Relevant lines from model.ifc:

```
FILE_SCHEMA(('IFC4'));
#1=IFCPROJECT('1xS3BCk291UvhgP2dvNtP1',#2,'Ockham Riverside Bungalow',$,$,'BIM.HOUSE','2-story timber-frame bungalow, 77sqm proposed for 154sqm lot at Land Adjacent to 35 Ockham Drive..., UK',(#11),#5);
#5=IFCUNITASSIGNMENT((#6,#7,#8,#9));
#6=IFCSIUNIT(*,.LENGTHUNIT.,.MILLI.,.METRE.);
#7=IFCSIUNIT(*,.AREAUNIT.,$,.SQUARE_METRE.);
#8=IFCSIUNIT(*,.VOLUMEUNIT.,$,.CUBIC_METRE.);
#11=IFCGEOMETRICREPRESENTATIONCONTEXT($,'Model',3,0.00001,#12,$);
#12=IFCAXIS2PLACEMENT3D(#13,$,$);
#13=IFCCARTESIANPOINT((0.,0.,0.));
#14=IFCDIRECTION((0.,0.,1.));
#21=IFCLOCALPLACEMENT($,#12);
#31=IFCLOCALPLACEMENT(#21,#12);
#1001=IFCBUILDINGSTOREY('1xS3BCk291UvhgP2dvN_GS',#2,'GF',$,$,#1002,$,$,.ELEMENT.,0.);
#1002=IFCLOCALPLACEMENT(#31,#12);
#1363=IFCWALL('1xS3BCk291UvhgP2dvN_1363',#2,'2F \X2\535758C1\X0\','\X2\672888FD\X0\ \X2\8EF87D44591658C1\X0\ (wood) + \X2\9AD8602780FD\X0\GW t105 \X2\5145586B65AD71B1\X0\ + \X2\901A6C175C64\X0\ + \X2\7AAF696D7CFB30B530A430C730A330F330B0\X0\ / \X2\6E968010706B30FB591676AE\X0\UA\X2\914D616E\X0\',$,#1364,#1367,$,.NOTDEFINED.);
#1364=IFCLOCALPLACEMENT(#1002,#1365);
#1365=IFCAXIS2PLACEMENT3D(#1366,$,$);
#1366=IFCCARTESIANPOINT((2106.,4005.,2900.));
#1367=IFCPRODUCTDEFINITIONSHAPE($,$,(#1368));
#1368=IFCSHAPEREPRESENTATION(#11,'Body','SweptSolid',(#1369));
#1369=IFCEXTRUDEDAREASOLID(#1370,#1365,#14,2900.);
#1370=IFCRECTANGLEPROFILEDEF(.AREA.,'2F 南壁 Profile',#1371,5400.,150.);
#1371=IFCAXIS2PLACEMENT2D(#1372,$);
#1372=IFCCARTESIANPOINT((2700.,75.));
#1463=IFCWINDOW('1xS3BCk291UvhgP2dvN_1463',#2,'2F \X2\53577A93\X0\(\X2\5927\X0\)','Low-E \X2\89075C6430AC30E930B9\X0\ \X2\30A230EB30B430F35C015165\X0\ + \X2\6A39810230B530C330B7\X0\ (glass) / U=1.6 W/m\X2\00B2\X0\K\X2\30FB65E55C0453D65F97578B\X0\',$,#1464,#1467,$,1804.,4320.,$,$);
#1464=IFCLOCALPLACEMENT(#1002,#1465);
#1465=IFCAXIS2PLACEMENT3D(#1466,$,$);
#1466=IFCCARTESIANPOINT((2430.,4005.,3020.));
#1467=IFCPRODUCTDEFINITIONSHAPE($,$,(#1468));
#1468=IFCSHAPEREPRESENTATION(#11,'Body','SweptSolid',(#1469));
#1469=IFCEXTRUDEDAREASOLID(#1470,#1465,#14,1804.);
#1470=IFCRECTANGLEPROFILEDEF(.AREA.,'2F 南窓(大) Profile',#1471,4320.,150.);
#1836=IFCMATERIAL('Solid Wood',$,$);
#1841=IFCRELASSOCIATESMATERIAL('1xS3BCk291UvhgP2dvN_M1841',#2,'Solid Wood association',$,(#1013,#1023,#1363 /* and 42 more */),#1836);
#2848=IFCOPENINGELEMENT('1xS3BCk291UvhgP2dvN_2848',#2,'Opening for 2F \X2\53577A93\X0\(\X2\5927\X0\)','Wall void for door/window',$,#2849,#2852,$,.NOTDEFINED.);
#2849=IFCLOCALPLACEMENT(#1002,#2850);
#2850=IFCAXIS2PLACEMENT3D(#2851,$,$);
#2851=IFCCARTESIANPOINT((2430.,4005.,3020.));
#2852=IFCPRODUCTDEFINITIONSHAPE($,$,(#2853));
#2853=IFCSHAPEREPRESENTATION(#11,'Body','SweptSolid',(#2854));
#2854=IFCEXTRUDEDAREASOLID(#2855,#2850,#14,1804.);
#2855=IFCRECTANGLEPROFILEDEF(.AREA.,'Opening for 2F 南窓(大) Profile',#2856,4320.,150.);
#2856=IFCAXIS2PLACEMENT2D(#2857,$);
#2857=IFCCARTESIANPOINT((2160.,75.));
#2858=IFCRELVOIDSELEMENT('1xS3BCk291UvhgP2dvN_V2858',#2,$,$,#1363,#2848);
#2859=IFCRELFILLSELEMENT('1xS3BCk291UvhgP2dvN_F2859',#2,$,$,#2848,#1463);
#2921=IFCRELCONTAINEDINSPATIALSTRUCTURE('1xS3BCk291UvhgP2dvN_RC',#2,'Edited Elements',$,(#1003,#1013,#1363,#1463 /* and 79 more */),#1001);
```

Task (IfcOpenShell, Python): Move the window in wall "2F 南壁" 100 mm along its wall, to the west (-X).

```python
import ifcopenshell
import ifcopenshell.api.geometry
import ifcopenshell.util.placement
import ifcopenshell.util.unit

model = ifcopenshell.open("model.ifc")
unit_scale = ifcopenshell.util.unit.calculate_unit_scale(model)

window = model.by_guid("1xS3BCk291UvhgP2dvN_1463")
opening = window.FillsVoids[0].RelatingOpeningElement
wall = opening.VoidsElements[0].RelatingBuildingElement

wall_matrix = ifcopenshell.util.placement.get_local_placement(wall.ObjectPlacement)
shift = wall_matrix[:3, 0] * -0.1 / unit_scale
before = ifcopenshell.util.placement.get_local_placement(window.ObjectPlacement)[:3, 3].copy()

# The window is not placed relative to its opening, so move both.
for product in (opening, window):
    matrix = ifcopenshell.util.placement.get_local_placement(product.ObjectPlacement)
    matrix[:3, 3] += shift
    ifcopenshell.api.geometry.edit_object_placement(model, product=product, matrix=matrix, is_si=False)

after = ifcopenshell.util.placement.get_local_placement(window.ObjectPlacement)[:3, 3]
print("window moved by", (after - before).round(3) + 0.0)

model.write("model_rev.ifc")
```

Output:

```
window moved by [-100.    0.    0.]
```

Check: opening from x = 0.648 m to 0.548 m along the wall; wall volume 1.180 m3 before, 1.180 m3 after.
